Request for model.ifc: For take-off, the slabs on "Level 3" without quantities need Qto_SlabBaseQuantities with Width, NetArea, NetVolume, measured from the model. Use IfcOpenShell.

First a look at what the model holds.

```python
import ifcopenshell
import ifcopenshell.util.element
import ifcopenshell.util.unit

model = ifcopenshell.open("model.ifc")
print(model.schema)
for unit_type in ("LENGTHUNIT", "AREAUNIT", "VOLUMEUNIT"):
    print(unit_type, ifcopenshell.util.unit.calculate_unit_scale(model, unit_type))
storey = next(s for s in model.by_type("IfcBuildingStorey") if s.Name == "Level 3")
slabs = [e for e in ifcopenshell.util.element.get_decomposition(storey) if e.is_a("IfcSlab")]
for e in sorted(slabs, key=lambda e: e.id()):
    print(e.id(), e.is_a(), e.Name, list(ifcopenshell.util.element.get_psets(e, qtos_only=True)), sep=" | ")
```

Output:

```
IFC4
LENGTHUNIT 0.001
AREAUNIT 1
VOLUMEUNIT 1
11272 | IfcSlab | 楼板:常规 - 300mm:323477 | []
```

```python
import ifcopenshell
import ifcopenshell.api.pset
import ifcopenshell.geom
import ifcopenshell.util.element
import ifcopenshell.util.shape
import ifcopenshell.util.unit

model = ifcopenshell.open("model.ifc")
unit_scale = ifcopenshell.util.unit.calculate_unit_scale(model)
area_scale = ifcopenshell.util.unit.calculate_unit_scale(model, "AREAUNIT")
volume_scale = ifcopenshell.util.unit.calculate_unit_scale(model, "VOLUMEUNIT")
settings = ifcopenshell.geom.settings()

storey = next(s for s in model.by_type("IfcBuildingStorey") if s.Name == "Level 3")
slabs = [e for e in ifcopenshell.util.element.get_decomposition(storey) if e.is_a("IfcSlab")]

for e in sorted(slabs, key=lambda e: e.id()):
    if ifcopenshell.util.element.get_psets(e, qtos_only=True, should_inherit=False):
        continue
    # Geometry comes back in metres, in the element's own axes.
    shape = ifcopenshell.geom.create_shape(settings, e)
    values = {
        "Width": ifcopenshell.util.shape.get_z(shape.geometry) / unit_scale,
        "NetArea": ifcopenshell.util.shape.get_footprint_area(shape.geometry) / area_scale,
        "NetVolume": ifcopenshell.util.shape.get_volume(shape.geometry) / volume_scale,
    }
    qto = ifcopenshell.api.pset.add_qto(model, product=e, name="Qto_SlabBaseQuantities")
    ifcopenshell.api.pset.edit_qto(model, qto=qto, properties=values)
    print(e.id(), {k: round(v, 3) for k, v in values.items()})

model.write("model_rev.ifc")
```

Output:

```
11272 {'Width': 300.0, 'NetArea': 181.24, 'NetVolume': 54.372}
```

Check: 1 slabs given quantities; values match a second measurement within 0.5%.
